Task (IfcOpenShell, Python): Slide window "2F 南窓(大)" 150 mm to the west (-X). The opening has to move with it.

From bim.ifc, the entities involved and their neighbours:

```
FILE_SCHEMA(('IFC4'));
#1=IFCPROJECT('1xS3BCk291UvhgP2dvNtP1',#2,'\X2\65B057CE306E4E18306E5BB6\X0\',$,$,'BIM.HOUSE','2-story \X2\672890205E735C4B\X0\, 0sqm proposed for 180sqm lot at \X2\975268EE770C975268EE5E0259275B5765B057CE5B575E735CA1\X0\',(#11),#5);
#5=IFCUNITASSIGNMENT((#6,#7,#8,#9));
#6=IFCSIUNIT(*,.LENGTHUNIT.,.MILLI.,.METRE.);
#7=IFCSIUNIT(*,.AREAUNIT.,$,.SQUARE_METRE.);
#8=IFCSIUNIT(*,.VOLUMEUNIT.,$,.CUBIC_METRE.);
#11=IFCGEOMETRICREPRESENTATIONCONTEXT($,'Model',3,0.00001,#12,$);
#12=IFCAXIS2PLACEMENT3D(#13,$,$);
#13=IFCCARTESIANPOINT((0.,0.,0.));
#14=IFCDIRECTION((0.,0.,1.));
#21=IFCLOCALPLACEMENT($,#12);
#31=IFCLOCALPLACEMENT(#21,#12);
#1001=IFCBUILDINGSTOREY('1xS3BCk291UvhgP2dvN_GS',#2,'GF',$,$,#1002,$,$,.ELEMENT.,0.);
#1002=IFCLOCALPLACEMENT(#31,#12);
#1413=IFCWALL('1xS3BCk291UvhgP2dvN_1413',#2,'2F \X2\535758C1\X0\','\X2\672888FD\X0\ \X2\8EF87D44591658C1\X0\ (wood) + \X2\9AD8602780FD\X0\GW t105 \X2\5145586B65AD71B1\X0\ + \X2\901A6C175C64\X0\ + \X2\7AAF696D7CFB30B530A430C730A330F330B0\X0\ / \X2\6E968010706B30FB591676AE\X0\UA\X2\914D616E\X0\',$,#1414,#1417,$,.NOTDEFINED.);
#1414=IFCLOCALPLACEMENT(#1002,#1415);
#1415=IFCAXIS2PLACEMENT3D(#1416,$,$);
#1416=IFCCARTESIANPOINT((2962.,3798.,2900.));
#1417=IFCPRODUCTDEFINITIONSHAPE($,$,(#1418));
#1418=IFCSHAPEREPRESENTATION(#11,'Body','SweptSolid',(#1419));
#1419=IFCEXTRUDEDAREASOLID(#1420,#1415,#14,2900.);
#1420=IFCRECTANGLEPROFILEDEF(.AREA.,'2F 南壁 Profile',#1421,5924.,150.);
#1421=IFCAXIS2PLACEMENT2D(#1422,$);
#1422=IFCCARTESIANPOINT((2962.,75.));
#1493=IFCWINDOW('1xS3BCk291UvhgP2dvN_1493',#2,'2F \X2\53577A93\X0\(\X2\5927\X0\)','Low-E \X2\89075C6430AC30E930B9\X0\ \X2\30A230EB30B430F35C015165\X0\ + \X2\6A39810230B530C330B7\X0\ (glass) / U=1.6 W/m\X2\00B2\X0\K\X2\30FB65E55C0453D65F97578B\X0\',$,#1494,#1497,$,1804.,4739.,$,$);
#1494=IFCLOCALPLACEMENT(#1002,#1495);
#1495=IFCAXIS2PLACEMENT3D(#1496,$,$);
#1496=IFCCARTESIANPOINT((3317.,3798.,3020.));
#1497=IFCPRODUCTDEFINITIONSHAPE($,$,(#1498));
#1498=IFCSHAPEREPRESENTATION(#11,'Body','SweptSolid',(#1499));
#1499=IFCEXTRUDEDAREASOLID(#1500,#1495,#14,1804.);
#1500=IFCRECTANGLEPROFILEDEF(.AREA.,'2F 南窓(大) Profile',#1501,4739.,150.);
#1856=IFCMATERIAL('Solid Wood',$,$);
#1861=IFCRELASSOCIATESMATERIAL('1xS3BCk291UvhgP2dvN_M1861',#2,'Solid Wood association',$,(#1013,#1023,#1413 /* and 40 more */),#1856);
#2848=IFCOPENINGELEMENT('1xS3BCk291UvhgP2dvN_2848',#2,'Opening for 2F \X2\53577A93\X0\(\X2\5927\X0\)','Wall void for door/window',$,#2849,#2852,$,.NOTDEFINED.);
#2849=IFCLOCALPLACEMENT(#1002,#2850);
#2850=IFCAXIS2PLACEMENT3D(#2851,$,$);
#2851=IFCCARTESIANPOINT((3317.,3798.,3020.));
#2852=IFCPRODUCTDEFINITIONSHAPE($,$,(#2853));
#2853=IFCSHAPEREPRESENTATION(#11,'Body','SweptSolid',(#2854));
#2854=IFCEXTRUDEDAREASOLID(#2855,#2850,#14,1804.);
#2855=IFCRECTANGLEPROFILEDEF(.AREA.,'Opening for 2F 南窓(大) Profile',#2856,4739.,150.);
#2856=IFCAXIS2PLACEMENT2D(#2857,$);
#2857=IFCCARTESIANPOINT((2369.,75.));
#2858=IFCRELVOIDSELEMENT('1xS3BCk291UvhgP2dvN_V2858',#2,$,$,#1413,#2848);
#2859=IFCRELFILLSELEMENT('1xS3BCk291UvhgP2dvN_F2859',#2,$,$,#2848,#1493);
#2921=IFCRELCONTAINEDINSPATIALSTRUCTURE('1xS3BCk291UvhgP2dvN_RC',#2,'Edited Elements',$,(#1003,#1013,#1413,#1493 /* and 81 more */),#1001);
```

```python
import ifcopenshell
import ifcopenshell.api.geometry
import ifcopenshell.util.placement
import ifcopenshell.util.unit

model = ifcopenshell.open("bim.ifc")
unit_scale = ifcopenshell.util.unit.calculate_unit_scale(model)

window = model.by_id(1493)
opening = window.FillsVoids[0].RelatingOpeningElement
wall = opening.VoidsElements[0].RelatingBuildingElement

wall_matrix = ifcopenshell.util.placement.get_local_placement(wall.ObjectPlacement)
shift = wall_matrix[:3, 0] * -0.15 / unit_scale
before = ifcopenshell.util.placement.get_local_placement(window.ObjectPlacement)[:3, 3].copy()

# The window is not placed relative to its opening, so move both.
for product in (opening, window):
    matrix = ifcopenshell.util.placement.get_local_placement(product.ObjectPlacement)
    matrix[:3, 3] += shift
    ifcopenshell.api.geometry.edit_object_placement(model, product=product, matrix=matrix, is_si=False)

after = ifcopenshell.util.placement.get_local_placement(window.ObjectPlacement)[:3, 3]
print("window moved by", (after - before).round(3) + 0.0)

model.write("bim_edited.ifc")
```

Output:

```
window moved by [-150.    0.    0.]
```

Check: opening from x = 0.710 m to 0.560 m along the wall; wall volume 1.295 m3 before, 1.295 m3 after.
